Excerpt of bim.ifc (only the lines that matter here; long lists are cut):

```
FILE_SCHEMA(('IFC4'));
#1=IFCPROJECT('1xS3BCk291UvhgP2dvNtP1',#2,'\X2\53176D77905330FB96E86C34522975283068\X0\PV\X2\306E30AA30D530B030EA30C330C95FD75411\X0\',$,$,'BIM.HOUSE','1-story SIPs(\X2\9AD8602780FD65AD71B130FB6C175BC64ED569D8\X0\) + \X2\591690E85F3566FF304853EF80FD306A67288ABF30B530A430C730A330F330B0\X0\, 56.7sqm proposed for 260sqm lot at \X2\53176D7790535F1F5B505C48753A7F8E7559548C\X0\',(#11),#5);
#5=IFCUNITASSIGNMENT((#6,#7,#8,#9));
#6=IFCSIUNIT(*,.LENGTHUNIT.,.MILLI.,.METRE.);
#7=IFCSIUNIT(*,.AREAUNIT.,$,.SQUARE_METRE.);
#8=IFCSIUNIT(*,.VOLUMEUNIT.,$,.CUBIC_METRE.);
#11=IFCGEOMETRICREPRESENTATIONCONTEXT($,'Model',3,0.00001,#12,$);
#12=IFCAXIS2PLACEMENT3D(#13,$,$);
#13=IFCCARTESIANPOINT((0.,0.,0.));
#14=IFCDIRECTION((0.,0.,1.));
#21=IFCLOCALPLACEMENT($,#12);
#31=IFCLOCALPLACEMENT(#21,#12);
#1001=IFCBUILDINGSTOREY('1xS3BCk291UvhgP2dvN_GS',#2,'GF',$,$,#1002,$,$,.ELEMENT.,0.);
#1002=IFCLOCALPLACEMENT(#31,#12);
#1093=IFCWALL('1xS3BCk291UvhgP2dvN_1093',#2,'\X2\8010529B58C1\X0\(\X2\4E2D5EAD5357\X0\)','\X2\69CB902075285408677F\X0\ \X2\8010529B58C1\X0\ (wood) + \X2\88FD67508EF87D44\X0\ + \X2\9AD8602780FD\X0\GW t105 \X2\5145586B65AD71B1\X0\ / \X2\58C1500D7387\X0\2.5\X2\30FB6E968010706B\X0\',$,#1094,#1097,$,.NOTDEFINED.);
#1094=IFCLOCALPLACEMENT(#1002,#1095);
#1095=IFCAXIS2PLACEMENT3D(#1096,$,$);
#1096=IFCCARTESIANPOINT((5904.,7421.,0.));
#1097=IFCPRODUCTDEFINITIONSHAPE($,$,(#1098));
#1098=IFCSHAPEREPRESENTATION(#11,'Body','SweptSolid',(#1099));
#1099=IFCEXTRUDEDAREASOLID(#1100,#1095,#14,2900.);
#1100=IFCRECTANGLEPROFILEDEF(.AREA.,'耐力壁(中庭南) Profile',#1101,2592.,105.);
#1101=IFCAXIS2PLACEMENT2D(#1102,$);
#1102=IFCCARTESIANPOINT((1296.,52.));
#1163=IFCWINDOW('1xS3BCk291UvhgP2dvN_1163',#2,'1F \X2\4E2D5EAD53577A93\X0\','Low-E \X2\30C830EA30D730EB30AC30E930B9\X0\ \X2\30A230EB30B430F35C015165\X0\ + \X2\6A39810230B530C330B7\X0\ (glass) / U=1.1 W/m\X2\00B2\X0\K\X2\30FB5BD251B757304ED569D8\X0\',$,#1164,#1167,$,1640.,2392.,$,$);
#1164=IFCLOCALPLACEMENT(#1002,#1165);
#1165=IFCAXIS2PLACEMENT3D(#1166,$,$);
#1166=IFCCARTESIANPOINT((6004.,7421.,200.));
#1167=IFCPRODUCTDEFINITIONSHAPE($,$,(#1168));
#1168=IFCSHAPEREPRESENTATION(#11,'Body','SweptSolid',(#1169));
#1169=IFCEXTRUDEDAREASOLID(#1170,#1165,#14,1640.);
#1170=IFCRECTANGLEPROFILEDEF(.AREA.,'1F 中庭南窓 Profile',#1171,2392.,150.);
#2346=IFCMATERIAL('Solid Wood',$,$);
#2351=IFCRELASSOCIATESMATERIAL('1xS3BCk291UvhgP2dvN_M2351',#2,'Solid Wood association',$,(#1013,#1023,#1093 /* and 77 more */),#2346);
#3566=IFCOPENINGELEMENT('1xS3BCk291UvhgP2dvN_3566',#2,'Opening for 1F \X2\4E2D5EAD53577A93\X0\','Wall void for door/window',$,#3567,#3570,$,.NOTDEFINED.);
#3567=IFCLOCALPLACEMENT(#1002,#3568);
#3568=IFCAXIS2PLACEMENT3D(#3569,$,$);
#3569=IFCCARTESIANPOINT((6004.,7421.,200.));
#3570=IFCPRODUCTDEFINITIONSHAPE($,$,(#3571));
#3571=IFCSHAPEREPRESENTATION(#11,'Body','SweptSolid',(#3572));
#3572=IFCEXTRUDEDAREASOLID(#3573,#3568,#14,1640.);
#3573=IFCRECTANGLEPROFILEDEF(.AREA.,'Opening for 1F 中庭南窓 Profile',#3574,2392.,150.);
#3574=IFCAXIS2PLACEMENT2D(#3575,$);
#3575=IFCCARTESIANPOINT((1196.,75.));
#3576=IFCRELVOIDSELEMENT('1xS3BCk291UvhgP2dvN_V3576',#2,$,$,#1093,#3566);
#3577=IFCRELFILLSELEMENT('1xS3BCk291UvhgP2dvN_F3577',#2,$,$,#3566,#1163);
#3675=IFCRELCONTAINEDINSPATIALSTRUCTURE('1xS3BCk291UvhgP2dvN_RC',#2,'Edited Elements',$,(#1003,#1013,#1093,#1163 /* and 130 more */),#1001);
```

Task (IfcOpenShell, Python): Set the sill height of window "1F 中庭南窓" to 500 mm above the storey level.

```python
import numpy as np
import ifcopenshell
import ifcopenshell.api.geometry
import ifcopenshell.geom
import ifcopenshell.util.element
import ifcopenshell.util.placement
import ifcopenshell.util.shape
import ifcopenshell.util.unit

model = ifcopenshell.open("bim.ifc")
unit_scale = ifcopenshell.util.unit.calculate_unit_scale(model)

window = model.by_guid("1xS3BCk291UvhgP2dvN_1163")
opening = window.FillsVoids[0].RelatingOpeningElement
storey = ifcopenshell.util.element.get_container(window, ifc_class="IfcBuildingStorey")
level = ifcopenshell.util.placement.get_local_placement(storey.ObjectPlacement)[2, 3]

# The opening's origin need not be at the sill, so measure its lowest point.
shape = ifcopenshell.geom.create_shape(ifcopenshell.geom.settings(), opening)
bottom = ifcopenshell.util.shape.get_shape_bottom_elevation(shape, shape.geometry) / unit_scale
dz = level + 500.0 - bottom

shift = np.array([0.0, 0.0, dz])
# The window is not placed relative to its opening, so move both.
for product in (opening, window):
    matrix = ifcopenshell.util.placement.get_local_placement(product.ObjectPlacement)
    matrix[:3, 3] += shift
    ifcopenshell.api.geometry.edit_object_placement(model, product=product, matrix=matrix, is_si=False)

print(f"moved by {dz * unit_scale:+.3f} m")

model.write("bim_updated.ifc")
```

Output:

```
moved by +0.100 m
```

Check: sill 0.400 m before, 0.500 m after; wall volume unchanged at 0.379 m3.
